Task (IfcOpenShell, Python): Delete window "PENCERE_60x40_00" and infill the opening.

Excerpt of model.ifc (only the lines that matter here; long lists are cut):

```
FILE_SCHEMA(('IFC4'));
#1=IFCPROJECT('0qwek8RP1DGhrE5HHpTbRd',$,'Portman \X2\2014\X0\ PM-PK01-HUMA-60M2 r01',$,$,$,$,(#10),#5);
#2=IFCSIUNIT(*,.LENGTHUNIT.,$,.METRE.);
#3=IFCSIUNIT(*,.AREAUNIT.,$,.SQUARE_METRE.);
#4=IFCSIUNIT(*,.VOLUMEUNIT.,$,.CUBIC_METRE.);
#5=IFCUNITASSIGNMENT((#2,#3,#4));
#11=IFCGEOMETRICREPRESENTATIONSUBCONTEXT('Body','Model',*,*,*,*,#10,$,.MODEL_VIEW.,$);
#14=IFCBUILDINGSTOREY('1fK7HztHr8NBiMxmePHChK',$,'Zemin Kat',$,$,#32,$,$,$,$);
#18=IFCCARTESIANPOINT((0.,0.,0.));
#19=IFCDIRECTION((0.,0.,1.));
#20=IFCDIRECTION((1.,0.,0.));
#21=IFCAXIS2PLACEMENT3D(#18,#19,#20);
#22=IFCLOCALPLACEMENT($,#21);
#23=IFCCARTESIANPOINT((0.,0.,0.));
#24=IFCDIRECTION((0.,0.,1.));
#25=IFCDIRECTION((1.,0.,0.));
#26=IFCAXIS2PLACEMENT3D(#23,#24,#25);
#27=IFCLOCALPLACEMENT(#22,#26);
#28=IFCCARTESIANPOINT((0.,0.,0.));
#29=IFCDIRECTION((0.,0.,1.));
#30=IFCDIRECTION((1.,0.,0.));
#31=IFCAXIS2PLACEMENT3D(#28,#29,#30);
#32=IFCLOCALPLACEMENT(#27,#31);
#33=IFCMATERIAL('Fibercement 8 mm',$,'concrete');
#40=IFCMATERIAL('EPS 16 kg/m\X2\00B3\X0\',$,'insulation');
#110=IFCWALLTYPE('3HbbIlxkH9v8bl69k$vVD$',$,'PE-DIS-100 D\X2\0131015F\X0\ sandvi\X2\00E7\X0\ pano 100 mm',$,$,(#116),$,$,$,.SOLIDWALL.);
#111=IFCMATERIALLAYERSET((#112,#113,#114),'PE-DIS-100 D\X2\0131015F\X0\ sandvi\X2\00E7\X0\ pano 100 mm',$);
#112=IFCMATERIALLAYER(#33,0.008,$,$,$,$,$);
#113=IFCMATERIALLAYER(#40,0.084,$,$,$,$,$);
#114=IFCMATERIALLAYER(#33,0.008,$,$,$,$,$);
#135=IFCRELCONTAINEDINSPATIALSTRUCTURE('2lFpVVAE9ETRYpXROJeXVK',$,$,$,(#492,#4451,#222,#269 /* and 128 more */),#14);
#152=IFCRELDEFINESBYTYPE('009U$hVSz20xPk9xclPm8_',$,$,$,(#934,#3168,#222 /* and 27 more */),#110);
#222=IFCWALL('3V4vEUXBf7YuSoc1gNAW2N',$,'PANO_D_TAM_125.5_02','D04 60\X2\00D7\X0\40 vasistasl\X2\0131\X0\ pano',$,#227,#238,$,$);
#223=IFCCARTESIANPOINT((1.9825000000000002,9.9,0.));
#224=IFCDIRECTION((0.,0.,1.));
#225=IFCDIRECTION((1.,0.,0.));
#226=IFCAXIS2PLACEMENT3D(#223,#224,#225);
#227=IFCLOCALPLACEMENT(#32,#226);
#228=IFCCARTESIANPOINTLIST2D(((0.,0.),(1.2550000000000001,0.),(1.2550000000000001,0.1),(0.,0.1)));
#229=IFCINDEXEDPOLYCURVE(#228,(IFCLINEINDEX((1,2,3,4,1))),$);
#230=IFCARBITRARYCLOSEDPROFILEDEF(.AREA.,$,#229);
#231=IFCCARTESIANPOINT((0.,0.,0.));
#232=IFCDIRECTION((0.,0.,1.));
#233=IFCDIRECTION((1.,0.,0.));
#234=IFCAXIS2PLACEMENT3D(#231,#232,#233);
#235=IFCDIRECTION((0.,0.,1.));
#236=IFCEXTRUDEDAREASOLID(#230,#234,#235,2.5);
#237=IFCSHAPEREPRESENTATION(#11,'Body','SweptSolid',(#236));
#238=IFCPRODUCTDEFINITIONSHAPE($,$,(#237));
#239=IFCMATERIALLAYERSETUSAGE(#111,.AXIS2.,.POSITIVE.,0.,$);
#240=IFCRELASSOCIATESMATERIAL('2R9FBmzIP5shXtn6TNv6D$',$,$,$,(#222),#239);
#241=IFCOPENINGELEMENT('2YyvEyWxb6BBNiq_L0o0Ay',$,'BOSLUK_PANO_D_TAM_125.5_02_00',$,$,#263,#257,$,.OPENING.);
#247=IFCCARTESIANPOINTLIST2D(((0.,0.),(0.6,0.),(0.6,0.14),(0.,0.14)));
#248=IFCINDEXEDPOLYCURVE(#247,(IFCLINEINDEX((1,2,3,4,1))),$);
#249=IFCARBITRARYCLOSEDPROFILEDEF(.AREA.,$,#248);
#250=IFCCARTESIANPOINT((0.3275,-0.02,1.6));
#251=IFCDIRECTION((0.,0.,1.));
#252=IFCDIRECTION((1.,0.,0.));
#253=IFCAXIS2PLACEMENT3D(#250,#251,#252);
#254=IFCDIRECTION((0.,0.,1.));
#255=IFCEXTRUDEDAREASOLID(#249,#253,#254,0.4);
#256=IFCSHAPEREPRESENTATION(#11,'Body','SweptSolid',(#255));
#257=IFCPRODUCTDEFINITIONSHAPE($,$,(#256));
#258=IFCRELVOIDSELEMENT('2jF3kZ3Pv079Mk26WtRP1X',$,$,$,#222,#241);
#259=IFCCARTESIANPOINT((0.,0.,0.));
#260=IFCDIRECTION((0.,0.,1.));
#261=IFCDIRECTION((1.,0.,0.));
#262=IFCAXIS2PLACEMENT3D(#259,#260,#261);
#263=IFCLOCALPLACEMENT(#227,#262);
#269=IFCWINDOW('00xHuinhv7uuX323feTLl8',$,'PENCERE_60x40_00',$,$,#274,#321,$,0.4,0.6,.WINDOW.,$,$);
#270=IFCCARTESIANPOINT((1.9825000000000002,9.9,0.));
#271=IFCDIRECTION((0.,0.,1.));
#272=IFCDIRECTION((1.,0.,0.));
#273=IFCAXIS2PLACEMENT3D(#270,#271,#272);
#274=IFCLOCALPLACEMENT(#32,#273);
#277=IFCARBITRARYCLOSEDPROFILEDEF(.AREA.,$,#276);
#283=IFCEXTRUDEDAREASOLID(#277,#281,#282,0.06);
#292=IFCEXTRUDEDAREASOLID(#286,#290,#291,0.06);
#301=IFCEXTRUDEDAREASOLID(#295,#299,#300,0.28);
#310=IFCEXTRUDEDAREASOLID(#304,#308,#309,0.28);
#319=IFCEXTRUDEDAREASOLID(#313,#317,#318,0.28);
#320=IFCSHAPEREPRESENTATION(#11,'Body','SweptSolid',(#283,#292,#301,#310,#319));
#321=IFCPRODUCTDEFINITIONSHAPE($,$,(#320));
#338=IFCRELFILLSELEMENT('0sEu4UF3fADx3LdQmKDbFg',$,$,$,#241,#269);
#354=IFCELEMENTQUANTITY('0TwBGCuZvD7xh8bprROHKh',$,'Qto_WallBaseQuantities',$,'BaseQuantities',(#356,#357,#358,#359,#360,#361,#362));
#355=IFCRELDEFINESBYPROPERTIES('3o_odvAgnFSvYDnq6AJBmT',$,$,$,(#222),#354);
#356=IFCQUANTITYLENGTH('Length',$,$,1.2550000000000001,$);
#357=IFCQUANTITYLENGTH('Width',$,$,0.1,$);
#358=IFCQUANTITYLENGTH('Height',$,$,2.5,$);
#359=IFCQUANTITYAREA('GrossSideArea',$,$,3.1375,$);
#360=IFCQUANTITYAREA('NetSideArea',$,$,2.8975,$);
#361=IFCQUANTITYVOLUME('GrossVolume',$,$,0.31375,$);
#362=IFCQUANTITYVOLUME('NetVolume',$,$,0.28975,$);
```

```python
import ifcopenshell
import ifcopenshell.api.feature
import ifcopenshell.api.pset
import ifcopenshell.api.root
import ifcopenshell.geom
import ifcopenshell.util.element
import ifcopenshell.util.shape
import ifcopenshell.util.unit

model = ifcopenshell.open("model.ifc")
area_scale = ifcopenshell.util.unit.calculate_unit_scale(model, "AREAUNIT")
volume_scale = ifcopenshell.util.unit.calculate_unit_scale(model, "VOLUMEUNIT")
settings = ifcopenshell.geom.settings()


def volume(element):
    """Net volume in cubic metres, openings subtracted."""
    shape = ifcopenshell.geom.create_shape(settings, element)
    return ifcopenshell.util.shape.get_volume(shape.geometry)


window = model.by_guid("00xHuinhv7uuX323feTLl8")
opening = window.FillsVoids[0].RelatingOpeningElement
wall = opening.VoidsElements[0].RelatingBuildingElement
before = volume(wall)

ifcopenshell.api.root.remove_product(model, product=window)
ifcopenshell.api.feature.remove_feature(model, feature=opening)

after = volume(wall)
thickness = 0.1  # wall thickness in metres

# Update the wall's stored quantities.
qto = model.by_id(ifcopenshell.util.element.get_pset(wall, "Qto_WallBaseQuantities", should_inherit=False)["id"])
ifcopenshell.api.pset.edit_qto(model, qto=qto, properties={
    "NetSideArea": after / thickness / area_scale,
    "NetVolume": after / volume_scale,
})

print(f"wall volume {before:.3f} -> {after:.3f} m3")

model.write("model_edited.ifc")
```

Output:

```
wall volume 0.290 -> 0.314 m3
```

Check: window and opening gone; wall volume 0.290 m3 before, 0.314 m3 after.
